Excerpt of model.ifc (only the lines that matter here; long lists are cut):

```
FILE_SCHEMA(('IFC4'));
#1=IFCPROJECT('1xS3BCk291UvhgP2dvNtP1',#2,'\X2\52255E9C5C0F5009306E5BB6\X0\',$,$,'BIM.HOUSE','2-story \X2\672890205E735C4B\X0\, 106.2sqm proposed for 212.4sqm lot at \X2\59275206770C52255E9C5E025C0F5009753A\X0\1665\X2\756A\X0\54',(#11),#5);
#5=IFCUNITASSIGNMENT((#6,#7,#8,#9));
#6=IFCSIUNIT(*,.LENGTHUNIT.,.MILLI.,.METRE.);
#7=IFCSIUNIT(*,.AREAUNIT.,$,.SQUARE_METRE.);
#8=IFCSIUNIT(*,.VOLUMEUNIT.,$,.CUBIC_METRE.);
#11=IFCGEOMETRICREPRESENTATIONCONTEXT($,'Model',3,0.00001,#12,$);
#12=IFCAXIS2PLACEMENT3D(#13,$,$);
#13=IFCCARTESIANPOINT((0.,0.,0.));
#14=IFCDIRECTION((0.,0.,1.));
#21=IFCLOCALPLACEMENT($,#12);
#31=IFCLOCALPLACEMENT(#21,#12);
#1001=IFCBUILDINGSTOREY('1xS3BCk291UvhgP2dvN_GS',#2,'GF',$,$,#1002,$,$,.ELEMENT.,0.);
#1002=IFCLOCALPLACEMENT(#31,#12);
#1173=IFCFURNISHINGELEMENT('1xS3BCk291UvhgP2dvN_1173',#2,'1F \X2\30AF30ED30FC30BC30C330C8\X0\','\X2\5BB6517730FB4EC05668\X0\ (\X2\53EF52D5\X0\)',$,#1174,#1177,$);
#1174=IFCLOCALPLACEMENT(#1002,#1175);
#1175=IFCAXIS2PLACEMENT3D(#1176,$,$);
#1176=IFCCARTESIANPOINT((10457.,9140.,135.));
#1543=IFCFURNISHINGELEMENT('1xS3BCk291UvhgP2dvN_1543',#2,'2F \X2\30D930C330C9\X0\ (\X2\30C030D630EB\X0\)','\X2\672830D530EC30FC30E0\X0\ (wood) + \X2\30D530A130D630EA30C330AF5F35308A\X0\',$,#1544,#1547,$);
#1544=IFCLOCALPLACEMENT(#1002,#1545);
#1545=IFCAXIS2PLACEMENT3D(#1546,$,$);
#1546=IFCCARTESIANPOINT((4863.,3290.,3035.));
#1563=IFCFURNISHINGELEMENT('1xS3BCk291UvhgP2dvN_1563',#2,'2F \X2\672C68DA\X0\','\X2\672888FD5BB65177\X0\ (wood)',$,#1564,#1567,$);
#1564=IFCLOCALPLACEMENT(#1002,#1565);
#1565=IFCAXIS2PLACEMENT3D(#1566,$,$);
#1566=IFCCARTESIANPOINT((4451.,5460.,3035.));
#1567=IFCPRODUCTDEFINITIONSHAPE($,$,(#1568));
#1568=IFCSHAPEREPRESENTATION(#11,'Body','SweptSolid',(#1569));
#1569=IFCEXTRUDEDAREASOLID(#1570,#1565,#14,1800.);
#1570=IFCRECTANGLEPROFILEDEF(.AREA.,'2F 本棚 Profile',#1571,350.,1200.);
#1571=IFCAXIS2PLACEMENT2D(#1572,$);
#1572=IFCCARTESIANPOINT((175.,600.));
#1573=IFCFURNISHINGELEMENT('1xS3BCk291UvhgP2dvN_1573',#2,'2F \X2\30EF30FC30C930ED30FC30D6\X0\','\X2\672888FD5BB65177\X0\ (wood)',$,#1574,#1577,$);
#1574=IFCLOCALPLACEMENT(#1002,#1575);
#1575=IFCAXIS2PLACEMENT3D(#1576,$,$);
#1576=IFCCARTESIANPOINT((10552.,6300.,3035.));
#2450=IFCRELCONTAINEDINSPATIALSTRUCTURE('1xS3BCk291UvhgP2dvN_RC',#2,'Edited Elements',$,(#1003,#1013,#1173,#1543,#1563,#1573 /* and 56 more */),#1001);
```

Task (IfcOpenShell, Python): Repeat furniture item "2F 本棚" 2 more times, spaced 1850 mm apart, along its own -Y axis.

```python
import ifcopenshell
import ifcopenshell.api.geometry
import ifcopenshell.api.root
import ifcopenshell.util.element
import ifcopenshell.util.placement

model = ifcopenshell.open("model.ifc")


def reuse_history(source, copy):
    """copy_class also copies each property set's owner history, people and application; keep the originals."""
    for rel in copy.IsDefinedBy:
        if rel.is_a("IfcRelDefinesByProperties") and (history := rel.RelatingPropertyDefinition.OwnerHistory):
            rel.RelatingPropertyDefinition.OwnerHistory = source.OwnerHistory
            ifcopenshell.util.element.remove_deep2(model, history)


source = model.by_guid("1xS3BCk291UvhgP2dvN_1563")
base = ifcopenshell.util.placement.get_local_placement(source.ObjectPlacement)
step = -base[:3, 1] * 1850.0

for i in range(1, 3):
    copy = ifcopenshell.api.root.copy_class(model, product=source)
    copy.Representation = ifcopenshell.util.element.copy_deep(
        model, source.Representation, exclude=["IfcGeometricRepresentationContext", "IfcRepresentationMap"]
    )
    reuse_history(source, copy)
    matrix = base.copy()
    matrix[:3, 3] += i * step
    print("added at", matrix[:3, 3].round(3) + 0.0)
    ifcopenshell.api.geometry.edit_object_placement(model, product=copy, matrix=matrix, is_si=False)

model.write("model_edited.ifc")
```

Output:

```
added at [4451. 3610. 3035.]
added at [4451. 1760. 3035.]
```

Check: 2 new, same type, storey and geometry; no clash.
